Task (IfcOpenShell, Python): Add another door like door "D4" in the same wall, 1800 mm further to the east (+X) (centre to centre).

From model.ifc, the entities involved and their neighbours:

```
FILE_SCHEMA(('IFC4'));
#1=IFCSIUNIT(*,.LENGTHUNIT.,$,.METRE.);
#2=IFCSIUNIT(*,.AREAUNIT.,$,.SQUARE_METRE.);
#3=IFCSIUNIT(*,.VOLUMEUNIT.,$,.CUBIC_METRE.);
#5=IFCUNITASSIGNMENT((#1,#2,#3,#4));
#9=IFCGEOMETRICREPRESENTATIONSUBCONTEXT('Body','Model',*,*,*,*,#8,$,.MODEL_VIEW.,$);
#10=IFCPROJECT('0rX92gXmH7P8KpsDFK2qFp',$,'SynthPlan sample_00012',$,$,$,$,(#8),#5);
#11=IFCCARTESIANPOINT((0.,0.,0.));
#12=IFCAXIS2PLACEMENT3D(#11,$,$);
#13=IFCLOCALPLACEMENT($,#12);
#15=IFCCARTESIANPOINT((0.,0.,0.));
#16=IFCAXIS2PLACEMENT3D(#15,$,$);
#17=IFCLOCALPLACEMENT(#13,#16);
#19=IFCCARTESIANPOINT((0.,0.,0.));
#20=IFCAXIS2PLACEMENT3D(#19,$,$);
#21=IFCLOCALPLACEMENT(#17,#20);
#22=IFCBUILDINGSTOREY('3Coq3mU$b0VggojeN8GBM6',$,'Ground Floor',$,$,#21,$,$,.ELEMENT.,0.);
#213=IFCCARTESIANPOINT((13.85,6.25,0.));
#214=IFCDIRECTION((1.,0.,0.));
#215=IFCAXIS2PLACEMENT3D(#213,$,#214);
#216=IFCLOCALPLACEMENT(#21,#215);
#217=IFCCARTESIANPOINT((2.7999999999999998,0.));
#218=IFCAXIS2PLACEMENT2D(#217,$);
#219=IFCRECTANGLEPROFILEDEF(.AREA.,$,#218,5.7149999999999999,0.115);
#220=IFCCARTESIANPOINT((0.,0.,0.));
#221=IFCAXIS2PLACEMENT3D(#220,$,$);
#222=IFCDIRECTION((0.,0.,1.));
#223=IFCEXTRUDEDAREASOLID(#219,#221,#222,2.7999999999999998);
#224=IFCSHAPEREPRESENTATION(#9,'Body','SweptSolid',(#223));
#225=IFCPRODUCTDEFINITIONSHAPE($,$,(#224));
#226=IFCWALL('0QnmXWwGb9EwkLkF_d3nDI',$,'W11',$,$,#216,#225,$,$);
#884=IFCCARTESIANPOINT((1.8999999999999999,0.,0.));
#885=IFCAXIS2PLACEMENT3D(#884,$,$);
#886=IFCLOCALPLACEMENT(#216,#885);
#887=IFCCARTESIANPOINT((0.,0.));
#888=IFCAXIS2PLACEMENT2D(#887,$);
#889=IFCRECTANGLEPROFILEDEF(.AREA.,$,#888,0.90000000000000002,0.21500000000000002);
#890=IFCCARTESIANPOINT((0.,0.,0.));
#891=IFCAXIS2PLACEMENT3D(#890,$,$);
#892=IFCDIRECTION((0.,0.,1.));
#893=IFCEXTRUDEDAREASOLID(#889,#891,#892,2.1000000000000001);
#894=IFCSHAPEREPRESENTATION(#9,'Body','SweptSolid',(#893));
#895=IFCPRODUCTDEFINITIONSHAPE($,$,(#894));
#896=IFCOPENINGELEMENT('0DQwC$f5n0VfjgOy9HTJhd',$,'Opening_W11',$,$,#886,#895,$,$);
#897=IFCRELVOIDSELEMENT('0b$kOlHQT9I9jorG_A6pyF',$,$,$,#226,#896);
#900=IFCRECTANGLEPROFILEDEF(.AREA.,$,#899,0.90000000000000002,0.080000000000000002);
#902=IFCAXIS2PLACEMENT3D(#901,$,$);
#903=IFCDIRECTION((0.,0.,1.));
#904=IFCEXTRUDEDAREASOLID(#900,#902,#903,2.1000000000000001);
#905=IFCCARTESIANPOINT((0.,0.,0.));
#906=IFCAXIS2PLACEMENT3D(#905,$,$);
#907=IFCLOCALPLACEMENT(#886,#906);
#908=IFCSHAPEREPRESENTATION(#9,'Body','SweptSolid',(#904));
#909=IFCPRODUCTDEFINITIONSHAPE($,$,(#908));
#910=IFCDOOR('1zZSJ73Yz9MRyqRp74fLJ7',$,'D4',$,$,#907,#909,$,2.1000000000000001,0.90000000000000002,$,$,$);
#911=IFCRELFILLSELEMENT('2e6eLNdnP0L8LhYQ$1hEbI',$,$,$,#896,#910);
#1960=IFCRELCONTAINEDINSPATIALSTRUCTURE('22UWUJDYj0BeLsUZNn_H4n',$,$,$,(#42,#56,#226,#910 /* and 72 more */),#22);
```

```python
import ifcopenshell
import ifcopenshell.api.feature
import ifcopenshell.api.geometry
import ifcopenshell.api.root
import ifcopenshell.geom
import ifcopenshell.util.element
import ifcopenshell.util.placement
import ifcopenshell.util.shape

model = ifcopenshell.open("model.ifc")
settings = ifcopenshell.geom.settings()


def volume(element):
    """Net volume in cubic metres, openings subtracted."""
    shape = ifcopenshell.geom.create_shape(settings, element)
    return ifcopenshell.util.shape.get_volume(shape.geometry)


door = model.by_id(910)
opening = door.FillsVoids[0].RelatingOpeningElement
wall = opening.VoidsElements[0].RelatingBuildingElement
before = volume(wall)
shift = ifcopenshell.util.placement.get_local_placement(wall.ObjectPlacement)[:3, 0] * 1.8

# copy_class copies the void relationship, type, container and properties, but no geometry.
new_opening = ifcopenshell.api.root.copy_class(model, product=opening)
new_opening.Representation = ifcopenshell.util.element.copy_deep(
    model, opening.Representation, exclude=["IfcGeometricRepresentationContext", "IfcRepresentationMap"]
)
new_door = ifcopenshell.api.root.copy_class(model, product=door)
new_door.Representation = ifcopenshell.util.element.copy_deep(
    model, door.Representation, exclude=["IfcGeometricRepresentationContext", "IfcRepresentationMap"]
)
ifcopenshell.api.feature.add_filling(model, opening=new_opening, element=new_door)

for old, new in ((opening, new_opening), (door, new_door)):
    matrix = ifcopenshell.util.placement.get_local_placement(old.ObjectPlacement)
    matrix[:3, 3] += shift
    ifcopenshell.api.geometry.edit_object_placement(model, product=new, matrix=matrix, is_si=False)

after = volume(wall)

print(f"wall volume {before:.3f} -> {after:.3f} m3")

model.write("model_v2.ifc")
```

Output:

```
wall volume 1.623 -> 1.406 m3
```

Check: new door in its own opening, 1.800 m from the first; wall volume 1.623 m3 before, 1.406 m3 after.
